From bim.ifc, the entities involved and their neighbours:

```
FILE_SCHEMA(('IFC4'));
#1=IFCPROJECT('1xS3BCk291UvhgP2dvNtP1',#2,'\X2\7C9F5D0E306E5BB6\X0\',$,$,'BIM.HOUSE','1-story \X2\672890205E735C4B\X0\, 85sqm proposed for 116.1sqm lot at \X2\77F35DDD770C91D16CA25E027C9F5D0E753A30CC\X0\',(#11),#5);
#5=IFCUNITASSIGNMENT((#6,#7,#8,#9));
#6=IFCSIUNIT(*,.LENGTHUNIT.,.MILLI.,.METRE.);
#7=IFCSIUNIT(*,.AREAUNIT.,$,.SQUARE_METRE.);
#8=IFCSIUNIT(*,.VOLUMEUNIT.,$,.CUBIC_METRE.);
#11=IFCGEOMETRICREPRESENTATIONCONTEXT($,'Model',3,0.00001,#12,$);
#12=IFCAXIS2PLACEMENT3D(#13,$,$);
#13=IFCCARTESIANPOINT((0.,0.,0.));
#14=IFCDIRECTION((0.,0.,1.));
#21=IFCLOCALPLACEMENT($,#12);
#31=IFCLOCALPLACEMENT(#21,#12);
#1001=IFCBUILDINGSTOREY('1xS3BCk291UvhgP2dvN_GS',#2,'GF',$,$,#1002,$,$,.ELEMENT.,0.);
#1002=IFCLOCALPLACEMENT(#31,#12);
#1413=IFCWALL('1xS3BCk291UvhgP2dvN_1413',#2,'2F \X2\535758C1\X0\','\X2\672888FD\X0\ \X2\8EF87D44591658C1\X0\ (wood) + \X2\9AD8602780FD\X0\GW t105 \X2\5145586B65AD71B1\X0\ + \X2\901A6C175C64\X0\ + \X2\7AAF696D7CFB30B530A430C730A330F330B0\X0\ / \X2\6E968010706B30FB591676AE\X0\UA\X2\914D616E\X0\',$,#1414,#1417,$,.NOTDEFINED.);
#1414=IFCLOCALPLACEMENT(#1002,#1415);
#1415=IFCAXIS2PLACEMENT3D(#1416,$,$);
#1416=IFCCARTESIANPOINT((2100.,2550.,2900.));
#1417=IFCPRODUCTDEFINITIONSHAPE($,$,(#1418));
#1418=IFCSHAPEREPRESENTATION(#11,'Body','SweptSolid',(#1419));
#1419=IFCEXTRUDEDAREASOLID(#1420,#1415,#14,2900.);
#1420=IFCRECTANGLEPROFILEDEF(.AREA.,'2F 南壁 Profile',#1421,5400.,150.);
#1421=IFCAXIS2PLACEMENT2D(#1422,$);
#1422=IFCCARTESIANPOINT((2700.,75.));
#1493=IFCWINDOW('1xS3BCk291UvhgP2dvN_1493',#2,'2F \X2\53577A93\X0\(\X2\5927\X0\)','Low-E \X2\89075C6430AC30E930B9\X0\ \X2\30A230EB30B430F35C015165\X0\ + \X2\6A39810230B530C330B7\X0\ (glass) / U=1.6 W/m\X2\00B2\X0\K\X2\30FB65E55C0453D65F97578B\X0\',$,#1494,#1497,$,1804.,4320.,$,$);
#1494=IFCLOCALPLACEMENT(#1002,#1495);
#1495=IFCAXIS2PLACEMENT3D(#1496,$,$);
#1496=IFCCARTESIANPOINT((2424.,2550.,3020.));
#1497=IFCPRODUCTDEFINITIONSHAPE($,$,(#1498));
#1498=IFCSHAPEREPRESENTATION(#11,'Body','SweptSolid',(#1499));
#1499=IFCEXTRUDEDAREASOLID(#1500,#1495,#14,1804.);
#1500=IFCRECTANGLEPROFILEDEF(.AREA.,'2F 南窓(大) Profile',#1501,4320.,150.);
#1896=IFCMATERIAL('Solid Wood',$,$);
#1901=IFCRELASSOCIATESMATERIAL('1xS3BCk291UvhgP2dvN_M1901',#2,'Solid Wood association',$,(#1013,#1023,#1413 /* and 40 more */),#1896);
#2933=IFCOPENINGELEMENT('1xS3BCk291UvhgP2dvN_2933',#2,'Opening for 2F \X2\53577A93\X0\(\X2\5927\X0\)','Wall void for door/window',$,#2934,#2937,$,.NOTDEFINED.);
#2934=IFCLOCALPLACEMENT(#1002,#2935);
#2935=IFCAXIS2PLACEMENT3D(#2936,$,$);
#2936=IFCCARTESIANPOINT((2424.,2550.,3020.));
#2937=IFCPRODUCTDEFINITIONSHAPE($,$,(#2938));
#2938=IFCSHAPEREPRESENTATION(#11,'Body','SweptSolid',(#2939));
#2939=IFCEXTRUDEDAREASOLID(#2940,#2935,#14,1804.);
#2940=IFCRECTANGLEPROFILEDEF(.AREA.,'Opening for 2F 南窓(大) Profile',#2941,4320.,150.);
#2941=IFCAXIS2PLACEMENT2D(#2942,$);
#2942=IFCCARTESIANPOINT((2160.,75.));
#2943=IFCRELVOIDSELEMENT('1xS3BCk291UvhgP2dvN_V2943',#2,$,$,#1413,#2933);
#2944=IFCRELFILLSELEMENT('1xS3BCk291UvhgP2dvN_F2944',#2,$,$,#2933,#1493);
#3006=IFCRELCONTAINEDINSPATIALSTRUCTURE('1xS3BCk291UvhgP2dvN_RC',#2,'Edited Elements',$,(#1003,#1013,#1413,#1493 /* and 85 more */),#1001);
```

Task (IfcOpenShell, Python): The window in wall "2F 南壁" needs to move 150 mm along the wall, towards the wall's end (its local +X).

```python
import ifcopenshell
import ifcopenshell.api.geometry
import ifcopenshell.util.placement
import ifcopenshell.util.unit

model = ifcopenshell.open("bim.ifc")
unit_scale = ifcopenshell.util.unit.calculate_unit_scale(model)

window = model.by_id(1493)
opening = window.FillsVoids[0].RelatingOpeningElement
wall = opening.VoidsElements[0].RelatingBuildingElement

wall_matrix = ifcopenshell.util.placement.get_local_placement(wall.ObjectPlacement)
shift = wall_matrix[:3, 0] * 0.15 / unit_scale
before = ifcopenshell.util.placement.get_local_placement(window.ObjectPlacement)[:3, 3].copy()

# The window is not placed relative to its opening, so move both.
for product in (opening, window):
    matrix = ifcopenshell.util.placement.get_local_placement(product.ObjectPlacement)
    matrix[:3, 3] += shift
    ifcopenshell.api.geometry.edit_object_placement(model, product=product, matrix=matrix, is_si=False)

after = ifcopenshell.util.placement.get_local_placement(window.ObjectPlacement)[:3, 3]
print("window moved by", (after - before).round(3) + 0.0)

model.write("bim_edited.ifc")
```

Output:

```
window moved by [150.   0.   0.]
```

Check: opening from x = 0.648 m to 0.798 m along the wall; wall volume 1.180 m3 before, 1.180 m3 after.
